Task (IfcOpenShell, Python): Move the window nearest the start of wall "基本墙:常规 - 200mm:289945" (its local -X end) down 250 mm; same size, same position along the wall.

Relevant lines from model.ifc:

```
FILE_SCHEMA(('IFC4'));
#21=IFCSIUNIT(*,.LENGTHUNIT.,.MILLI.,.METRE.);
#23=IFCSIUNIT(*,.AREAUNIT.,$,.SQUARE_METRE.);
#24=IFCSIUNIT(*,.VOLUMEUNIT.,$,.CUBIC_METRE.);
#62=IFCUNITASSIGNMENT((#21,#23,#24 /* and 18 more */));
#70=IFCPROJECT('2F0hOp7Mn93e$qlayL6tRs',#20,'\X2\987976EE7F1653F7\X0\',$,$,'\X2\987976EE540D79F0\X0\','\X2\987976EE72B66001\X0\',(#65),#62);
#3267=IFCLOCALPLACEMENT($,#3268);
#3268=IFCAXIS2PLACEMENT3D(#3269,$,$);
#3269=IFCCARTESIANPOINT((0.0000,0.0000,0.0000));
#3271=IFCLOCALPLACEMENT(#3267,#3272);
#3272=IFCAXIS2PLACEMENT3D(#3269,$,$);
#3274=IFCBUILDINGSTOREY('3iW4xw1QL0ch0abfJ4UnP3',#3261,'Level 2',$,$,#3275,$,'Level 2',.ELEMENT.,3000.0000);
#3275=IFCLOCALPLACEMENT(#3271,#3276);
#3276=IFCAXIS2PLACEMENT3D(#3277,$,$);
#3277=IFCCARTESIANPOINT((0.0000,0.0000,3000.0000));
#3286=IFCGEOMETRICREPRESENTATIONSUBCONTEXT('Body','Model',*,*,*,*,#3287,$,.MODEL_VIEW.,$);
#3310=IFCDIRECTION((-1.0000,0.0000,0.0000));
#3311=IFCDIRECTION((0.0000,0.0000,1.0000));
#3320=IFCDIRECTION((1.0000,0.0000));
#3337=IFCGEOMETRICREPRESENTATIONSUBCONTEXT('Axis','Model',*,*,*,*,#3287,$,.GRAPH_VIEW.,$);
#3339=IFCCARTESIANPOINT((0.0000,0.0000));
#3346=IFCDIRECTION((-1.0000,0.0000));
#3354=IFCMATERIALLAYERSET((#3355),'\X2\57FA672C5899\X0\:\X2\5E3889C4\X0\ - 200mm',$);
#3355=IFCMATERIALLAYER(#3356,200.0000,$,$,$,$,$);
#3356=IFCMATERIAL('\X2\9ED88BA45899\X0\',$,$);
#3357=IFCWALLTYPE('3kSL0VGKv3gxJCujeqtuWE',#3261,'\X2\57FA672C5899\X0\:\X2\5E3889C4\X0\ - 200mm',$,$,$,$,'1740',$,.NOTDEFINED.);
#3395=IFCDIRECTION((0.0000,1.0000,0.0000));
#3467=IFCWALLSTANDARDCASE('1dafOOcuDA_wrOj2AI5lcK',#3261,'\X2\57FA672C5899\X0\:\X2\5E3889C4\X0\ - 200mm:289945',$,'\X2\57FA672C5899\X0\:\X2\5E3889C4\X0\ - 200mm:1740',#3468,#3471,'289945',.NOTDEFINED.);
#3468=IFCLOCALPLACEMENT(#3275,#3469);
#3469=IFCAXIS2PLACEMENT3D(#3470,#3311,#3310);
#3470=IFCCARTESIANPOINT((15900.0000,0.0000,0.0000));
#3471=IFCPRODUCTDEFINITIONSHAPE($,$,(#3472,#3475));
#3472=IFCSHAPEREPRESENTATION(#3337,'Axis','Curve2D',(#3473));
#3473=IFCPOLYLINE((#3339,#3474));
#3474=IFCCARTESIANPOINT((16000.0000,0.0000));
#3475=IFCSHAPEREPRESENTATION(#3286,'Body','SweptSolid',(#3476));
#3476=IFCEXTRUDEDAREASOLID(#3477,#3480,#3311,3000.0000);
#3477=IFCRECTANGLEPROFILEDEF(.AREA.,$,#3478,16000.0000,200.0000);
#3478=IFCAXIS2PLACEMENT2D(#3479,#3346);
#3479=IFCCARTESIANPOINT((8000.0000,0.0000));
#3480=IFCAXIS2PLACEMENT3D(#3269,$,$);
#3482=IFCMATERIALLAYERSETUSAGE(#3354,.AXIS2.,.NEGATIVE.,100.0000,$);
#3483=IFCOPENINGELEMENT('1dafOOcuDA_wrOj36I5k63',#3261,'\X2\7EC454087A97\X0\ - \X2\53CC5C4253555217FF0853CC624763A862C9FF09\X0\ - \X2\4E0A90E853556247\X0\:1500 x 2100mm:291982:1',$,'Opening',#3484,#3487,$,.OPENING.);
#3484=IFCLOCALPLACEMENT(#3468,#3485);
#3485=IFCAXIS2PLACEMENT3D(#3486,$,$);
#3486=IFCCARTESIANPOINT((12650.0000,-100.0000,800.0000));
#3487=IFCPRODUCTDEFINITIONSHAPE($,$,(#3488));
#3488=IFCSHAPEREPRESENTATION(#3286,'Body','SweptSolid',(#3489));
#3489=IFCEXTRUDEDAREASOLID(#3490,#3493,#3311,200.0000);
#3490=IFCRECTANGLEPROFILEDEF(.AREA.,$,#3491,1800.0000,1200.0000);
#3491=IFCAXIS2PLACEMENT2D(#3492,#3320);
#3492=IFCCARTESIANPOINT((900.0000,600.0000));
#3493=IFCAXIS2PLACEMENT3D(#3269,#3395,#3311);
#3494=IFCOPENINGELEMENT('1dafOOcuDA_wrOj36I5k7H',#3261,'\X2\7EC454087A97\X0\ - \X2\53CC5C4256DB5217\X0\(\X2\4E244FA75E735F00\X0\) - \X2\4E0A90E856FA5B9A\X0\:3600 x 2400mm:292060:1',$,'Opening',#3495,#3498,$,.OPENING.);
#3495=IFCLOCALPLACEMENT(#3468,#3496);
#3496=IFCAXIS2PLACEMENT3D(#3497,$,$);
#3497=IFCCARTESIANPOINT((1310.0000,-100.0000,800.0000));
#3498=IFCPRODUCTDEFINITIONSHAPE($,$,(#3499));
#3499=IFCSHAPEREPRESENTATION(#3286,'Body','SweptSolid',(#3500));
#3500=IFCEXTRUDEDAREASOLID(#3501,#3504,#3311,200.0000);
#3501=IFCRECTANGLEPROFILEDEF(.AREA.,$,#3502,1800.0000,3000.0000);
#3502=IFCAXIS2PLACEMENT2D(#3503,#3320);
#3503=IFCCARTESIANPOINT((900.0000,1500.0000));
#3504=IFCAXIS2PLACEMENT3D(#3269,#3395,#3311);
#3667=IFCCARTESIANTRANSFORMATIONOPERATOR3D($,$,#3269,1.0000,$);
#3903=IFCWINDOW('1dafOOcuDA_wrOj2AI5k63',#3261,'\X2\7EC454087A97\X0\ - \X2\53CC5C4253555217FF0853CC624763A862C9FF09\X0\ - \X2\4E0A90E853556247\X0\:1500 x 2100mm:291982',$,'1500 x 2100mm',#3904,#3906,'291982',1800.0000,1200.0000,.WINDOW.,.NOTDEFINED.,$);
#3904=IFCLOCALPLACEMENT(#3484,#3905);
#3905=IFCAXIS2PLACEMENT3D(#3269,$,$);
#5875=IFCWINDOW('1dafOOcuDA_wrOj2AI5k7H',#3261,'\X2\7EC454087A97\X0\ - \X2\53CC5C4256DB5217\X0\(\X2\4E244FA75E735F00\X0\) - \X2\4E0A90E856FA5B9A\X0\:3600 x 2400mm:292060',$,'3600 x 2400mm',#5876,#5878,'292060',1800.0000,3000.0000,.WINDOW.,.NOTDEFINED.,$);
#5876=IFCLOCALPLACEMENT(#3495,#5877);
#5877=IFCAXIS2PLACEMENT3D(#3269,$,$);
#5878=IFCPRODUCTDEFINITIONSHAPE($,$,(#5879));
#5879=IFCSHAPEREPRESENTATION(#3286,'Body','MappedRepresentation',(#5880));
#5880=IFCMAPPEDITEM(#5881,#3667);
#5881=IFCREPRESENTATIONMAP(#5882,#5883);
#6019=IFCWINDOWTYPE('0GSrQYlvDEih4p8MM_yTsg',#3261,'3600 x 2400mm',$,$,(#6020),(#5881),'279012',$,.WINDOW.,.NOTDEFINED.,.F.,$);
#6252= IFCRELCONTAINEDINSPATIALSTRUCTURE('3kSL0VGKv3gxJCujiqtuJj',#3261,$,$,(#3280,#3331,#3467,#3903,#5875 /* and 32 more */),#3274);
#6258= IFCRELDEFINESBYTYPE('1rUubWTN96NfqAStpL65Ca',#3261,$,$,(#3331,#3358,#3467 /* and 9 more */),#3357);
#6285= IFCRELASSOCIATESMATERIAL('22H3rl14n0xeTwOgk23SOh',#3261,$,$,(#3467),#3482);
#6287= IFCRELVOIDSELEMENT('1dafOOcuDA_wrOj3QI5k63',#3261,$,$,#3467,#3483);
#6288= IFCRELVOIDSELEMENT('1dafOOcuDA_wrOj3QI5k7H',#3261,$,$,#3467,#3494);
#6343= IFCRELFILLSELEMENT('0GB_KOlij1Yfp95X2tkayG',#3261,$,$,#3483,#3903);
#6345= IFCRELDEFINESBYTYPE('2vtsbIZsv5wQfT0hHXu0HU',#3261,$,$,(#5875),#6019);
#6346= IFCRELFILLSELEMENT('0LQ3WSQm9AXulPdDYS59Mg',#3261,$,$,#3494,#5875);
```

```python
import numpy as np
import ifcopenshell
import ifcopenshell.api.geometry
import ifcopenshell.util.placement
import ifcopenshell.util.unit

model = ifcopenshell.open("model.ifc")
unit_scale = ifcopenshell.util.unit.calculate_unit_scale(model)

window = model.by_guid("1dafOOcuDA_wrOj2AI5k7H")
opening = window.FillsVoids[0].RelatingOpeningElement
dz = -0.25 / unit_scale

shift = np.array([0.0, 0.0, dz])
# The window is placed relative to its opening, so it follows when the opening moves.
matrix = ifcopenshell.util.placement.get_local_placement(opening.ObjectPlacement)
matrix[:3, 3] += shift
ifcopenshell.api.geometry.edit_object_placement(
    model, product=opening, matrix=matrix, is_si=False, should_transform_children=True
)

print(f"moved by {dz * unit_scale:+.3f} m")

model.write("model_rev.ifc")
```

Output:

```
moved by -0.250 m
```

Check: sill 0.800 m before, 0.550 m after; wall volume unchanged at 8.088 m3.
